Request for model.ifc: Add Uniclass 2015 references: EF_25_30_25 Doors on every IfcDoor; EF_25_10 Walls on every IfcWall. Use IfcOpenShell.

First a look at what the model holds.

```python
import ifcopenshell

model = ifcopenshell.open("model.ifc")
print(model.schema)
print("classifications:", [c.Name for c in model.by_type("IfcClassification")])
for ifc_class in ("IfcDoor", "IfcRoof", "IfcStair", "IfcWall", "IfcWindow"):
    print(ifc_class, len(model.by_type(ifc_class)))
```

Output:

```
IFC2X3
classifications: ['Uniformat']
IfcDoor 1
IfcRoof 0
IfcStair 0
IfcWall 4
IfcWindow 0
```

```python
import ifcopenshell
import ifcopenshell.api.classification

model = ifcopenshell.open("model.ifc")

# IFC2X3 requires Source and Edition and has no link from the project to the system.
system = model.create_entity("IfcClassification", Source="NBS", Edition="2015", Name="Uniclass 2015")

codes = {
    "IfcDoor": ("EF_25_30_25", "Doors"),
    "IfcWall": ("EF_25_10", "Walls"),
}
for ifc_class, (code, name) in codes.items():
    products = model.by_type(ifc_class)
    ifcopenshell.api.classification.add_reference(
        model, products=products, classification=system, identification=code, name=name
    )
    print(code, len(products))

model.write("model_edited.ifc")
```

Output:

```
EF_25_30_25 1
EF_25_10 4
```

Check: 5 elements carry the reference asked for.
